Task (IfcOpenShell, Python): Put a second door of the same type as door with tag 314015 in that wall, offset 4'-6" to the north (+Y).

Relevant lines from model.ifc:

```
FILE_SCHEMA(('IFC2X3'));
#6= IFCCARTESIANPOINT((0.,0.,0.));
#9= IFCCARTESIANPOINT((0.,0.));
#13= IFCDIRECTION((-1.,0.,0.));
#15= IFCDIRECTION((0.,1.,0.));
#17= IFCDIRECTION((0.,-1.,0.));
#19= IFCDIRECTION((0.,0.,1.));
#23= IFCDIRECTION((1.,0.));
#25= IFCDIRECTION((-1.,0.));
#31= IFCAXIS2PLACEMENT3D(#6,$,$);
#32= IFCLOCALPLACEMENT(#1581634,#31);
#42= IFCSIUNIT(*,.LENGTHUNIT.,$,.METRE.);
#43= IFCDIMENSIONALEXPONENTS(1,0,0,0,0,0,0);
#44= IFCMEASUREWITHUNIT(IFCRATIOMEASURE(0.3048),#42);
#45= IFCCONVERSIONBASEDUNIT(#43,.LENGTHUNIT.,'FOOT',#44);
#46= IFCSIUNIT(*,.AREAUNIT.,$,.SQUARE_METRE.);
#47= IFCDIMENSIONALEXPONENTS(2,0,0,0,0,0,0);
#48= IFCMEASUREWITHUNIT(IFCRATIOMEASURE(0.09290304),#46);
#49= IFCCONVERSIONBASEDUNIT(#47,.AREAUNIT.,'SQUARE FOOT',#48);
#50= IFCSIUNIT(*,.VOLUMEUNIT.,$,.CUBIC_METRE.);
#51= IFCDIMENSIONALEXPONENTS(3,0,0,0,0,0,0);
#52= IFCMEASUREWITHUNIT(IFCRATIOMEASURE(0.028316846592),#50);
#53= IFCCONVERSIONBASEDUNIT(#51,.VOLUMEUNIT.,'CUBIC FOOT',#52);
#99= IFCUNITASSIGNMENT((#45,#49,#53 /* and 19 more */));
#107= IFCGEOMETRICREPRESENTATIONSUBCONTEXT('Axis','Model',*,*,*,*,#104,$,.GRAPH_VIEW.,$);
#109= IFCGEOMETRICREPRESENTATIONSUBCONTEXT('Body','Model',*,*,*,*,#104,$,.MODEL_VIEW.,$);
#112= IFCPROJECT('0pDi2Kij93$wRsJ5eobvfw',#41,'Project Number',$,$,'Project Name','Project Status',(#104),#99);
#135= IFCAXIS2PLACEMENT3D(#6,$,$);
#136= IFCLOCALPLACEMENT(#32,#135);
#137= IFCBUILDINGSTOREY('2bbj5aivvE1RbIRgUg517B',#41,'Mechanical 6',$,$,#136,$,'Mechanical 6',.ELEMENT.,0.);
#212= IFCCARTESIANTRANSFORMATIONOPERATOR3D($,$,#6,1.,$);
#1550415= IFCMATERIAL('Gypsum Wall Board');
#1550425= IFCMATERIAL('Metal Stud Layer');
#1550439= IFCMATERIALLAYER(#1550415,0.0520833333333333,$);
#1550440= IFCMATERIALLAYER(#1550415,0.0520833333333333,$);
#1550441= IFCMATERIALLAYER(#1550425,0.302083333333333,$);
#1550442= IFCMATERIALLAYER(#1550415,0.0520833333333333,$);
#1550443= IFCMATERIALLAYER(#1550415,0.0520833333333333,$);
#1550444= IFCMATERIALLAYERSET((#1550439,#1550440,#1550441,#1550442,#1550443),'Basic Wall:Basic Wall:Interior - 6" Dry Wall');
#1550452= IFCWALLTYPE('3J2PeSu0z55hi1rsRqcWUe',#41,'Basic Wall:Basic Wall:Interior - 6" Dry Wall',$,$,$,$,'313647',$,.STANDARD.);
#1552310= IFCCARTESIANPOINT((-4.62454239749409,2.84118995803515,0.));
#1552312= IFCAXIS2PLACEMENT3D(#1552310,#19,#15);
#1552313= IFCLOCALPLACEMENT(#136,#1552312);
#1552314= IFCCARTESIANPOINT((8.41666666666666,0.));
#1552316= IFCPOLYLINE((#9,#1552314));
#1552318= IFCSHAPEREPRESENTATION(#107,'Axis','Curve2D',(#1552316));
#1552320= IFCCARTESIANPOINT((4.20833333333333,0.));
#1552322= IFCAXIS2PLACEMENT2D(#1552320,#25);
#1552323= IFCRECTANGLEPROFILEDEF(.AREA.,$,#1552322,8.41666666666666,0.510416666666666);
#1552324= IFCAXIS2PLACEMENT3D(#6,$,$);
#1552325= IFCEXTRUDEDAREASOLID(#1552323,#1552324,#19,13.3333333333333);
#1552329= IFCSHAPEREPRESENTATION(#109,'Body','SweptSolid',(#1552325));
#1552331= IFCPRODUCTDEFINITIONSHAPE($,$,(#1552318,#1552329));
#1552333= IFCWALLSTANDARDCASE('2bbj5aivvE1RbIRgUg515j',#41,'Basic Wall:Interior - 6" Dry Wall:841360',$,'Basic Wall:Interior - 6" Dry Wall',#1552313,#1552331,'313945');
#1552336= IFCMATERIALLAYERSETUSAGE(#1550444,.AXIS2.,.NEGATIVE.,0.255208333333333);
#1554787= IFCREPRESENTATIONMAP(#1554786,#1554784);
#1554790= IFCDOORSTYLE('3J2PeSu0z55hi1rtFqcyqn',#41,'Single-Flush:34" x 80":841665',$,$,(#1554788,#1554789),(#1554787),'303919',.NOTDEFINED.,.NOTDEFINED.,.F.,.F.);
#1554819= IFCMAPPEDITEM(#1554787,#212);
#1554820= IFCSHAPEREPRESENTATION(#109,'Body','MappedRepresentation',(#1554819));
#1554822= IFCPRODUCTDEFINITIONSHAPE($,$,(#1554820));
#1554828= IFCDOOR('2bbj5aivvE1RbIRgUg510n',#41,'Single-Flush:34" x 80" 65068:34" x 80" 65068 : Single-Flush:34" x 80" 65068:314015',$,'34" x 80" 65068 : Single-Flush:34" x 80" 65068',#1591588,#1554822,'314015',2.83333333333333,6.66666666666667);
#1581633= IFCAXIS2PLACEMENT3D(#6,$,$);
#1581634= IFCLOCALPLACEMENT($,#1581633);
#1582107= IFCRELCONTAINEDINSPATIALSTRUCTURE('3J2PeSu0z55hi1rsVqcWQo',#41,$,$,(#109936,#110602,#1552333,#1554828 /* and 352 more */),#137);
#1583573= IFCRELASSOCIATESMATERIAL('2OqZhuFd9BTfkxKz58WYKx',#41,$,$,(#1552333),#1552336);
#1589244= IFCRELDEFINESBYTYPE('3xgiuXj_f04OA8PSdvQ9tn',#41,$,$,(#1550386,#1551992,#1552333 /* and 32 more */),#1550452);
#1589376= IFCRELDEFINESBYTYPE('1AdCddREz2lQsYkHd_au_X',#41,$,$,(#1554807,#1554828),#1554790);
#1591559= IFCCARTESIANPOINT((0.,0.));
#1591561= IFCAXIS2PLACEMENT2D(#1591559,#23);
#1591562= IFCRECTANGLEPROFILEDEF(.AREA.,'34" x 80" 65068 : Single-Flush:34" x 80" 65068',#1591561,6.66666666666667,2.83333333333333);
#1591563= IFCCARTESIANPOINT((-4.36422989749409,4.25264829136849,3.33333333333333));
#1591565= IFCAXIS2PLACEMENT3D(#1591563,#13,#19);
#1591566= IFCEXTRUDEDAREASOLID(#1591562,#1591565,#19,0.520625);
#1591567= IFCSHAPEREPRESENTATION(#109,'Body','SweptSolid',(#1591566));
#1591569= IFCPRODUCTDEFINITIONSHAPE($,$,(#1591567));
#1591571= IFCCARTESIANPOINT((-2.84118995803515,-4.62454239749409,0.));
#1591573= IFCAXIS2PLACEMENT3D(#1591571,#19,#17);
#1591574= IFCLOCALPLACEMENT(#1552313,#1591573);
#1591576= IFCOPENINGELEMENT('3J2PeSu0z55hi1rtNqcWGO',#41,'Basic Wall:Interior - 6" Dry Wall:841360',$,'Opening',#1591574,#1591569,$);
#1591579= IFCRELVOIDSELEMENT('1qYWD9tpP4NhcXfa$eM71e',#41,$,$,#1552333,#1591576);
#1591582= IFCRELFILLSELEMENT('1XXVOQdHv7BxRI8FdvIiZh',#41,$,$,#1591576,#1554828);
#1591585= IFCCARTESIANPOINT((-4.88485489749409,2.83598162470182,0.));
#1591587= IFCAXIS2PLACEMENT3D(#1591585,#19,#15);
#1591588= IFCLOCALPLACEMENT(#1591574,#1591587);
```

```python
import ifcopenshell
import ifcopenshell.api.feature
import ifcopenshell.api.geometry
import ifcopenshell.api.root
import ifcopenshell.geom
import ifcopenshell.util.element
import ifcopenshell.util.placement
import ifcopenshell.util.shape
import ifcopenshell.util.unit

model = ifcopenshell.open("model.ifc")
unit_scale = ifcopenshell.util.unit.calculate_unit_scale(model)
settings = ifcopenshell.geom.settings()


def volume(element):
    """Net volume in cubic metres, openings subtracted."""
    shape = ifcopenshell.geom.create_shape(settings, element)
    return ifcopenshell.util.shape.get_volume(shape.geometry)


def reuse_history(source, copy):
    """copy_class also copies each property set's owner history, people and application; keep the originals."""
    for rel in copy.IsDefinedBy:
        if rel.is_a("IfcRelDefinesByProperties") and (history := rel.RelatingPropertyDefinition.OwnerHistory):
            rel.RelatingPropertyDefinition.OwnerHistory = source.OwnerHistory
            ifcopenshell.util.element.remove_deep2(model, history)


door = model.by_guid("2bbj5aivvE1RbIRgUg510n")
opening = door.FillsVoids[0].RelatingOpeningElement
wall = opening.VoidsElements[0].RelatingBuildingElement
before = volume(wall)
shift = ifcopenshell.util.placement.get_local_placement(wall.ObjectPlacement)[:3, 0] * 54 * 0.0254 / unit_scale

# copy_class copies the void relationship, type, container and properties, but no geometry.
new_opening = ifcopenshell.api.root.copy_class(model, product=opening)
new_opening.Representation = ifcopenshell.util.element.copy_deep(
    model, opening.Representation, exclude=["IfcGeometricRepresentationContext", "IfcRepresentationMap"]
)
new_opening.Name = 'Basic Wall:Interior - 6" Dry Wall'
new_door = ifcopenshell.api.root.copy_class(model, product=door)
new_door.Representation = ifcopenshell.util.element.copy_deep(
    model, door.Representation, exclude=["IfcGeometricRepresentationContext", "IfcRepresentationMap"]
)
new_door.Name = 'Single-Flush:34" x 80" 65068:34" x 80" 65068 : Single-Flush:34" x 80" 65068'
new_door.Tag = None
reuse_history(door, new_door)
fills = ifcopenshell.api.feature.add_filling(model, opening=new_opening, element=new_door)
fills.OwnerHistory = new_door.OwnerHistory  # required in IFC2X3

for old, new in ((opening, new_opening), (door, new_door)):
    matrix = ifcopenshell.util.placement.get_local_placement(old.ObjectPlacement)
    matrix[:3, 3] += shift
    ifcopenshell.api.geometry.edit_object_placement(model, product=new, matrix=matrix, is_si=False)

after = volume(wall)

print(f"wall volume {before:.3f} -> {after:.3f} m3")

model.write("model_rev.ifc")
```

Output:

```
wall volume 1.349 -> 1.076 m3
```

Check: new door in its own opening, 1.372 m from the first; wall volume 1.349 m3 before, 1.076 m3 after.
